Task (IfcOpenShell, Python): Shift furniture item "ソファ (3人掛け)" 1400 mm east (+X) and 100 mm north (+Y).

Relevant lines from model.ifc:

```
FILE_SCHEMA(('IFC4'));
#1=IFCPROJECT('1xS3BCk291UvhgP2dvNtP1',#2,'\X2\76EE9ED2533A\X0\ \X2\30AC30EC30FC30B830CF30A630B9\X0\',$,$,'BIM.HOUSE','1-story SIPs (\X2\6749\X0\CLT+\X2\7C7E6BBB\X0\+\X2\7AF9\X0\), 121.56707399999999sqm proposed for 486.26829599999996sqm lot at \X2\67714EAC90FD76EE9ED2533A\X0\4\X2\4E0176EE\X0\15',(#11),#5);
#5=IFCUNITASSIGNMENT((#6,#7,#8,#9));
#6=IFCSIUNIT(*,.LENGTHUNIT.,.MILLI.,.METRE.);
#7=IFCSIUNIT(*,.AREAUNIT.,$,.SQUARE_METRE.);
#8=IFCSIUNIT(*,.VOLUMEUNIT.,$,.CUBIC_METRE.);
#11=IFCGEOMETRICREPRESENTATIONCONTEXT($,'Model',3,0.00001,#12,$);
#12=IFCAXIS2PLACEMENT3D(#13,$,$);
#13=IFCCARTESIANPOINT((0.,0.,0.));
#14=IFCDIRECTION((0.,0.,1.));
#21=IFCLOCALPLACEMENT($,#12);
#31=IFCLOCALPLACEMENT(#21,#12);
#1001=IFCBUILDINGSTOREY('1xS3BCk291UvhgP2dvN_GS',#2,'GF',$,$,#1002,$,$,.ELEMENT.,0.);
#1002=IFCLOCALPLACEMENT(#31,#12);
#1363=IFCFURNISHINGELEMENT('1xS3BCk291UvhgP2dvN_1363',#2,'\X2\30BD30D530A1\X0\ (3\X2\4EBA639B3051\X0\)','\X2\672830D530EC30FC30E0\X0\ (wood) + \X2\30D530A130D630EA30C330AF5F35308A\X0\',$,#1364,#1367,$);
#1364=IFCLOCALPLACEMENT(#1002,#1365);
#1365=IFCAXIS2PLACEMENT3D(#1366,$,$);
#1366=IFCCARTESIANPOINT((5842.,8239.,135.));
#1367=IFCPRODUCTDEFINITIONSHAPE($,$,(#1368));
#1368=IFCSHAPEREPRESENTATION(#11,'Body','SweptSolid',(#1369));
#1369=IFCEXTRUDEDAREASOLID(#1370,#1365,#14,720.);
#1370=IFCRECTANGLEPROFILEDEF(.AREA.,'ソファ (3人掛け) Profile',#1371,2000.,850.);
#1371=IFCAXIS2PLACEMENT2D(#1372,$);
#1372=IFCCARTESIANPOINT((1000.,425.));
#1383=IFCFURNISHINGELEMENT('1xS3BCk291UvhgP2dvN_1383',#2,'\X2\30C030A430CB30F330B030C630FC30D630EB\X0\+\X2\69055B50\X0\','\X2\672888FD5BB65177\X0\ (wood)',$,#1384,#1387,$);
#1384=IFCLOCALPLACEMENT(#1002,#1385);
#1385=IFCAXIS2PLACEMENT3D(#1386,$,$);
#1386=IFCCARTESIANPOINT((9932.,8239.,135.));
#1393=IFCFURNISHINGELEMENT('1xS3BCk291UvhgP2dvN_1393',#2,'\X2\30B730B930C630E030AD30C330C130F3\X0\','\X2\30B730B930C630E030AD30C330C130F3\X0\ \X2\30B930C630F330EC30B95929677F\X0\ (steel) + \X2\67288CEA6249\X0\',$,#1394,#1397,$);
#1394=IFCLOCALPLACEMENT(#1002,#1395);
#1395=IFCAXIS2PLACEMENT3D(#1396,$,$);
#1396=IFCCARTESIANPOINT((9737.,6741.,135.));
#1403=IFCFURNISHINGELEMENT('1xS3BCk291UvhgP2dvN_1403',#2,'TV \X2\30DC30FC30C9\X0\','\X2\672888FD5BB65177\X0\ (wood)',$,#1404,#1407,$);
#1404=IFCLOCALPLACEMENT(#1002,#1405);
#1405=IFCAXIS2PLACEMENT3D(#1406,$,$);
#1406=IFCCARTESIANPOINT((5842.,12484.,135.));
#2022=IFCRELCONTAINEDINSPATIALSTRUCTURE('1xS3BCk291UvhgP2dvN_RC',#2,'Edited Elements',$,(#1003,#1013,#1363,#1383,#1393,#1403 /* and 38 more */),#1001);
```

```python
import ifcopenshell
import ifcopenshell.api.geometry
import ifcopenshell.util.placement

model = ifcopenshell.open("model.ifc")

item = model.by_id(1363)
matrix = ifcopenshell.util.placement.get_local_placement(item.ObjectPlacement)
matrix[0, 3] += 1400.0
matrix[1, 3] += 100.0
ifcopenshell.api.geometry.edit_object_placement(model, product=item, matrix=matrix, is_si=False)

print(ifcopenshell.util.placement.get_local_placement(item.ObjectPlacement).round(3) + 0.0)

model.write("model_v2.ifc")
```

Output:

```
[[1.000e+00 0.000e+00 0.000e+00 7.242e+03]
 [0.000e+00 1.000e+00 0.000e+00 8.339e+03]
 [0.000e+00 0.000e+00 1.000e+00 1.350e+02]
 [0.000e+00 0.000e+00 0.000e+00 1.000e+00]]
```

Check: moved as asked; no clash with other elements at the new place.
